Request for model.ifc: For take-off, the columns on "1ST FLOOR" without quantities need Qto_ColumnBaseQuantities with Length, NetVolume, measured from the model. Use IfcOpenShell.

First a look at what the model holds.

```python
import ifcopenshell
import ifcopenshell.util.element
import ifcopenshell.util.unit

model = ifcopenshell.open("model.ifc")
print(model.schema)
for unit_type in ("LENGTHUNIT", "AREAUNIT", "VOLUMEUNIT"):
    print(unit_type, ifcopenshell.util.unit.calculate_unit_scale(model, unit_type))
storey = next(s for s in model.by_type("IfcBuildingStorey") if s.Name == "1ST FLOOR")
columns = [e for e in ifcopenshell.util.element.get_decomposition(storey) if e.is_a("IfcColumn")]
for e in sorted(columns, key=lambda e: e.id()):
    print(e.id(), e.is_a(), e.Name, list(ifcopenshell.util.element.get_psets(e, qtos_only=True)), sep=" | ")
```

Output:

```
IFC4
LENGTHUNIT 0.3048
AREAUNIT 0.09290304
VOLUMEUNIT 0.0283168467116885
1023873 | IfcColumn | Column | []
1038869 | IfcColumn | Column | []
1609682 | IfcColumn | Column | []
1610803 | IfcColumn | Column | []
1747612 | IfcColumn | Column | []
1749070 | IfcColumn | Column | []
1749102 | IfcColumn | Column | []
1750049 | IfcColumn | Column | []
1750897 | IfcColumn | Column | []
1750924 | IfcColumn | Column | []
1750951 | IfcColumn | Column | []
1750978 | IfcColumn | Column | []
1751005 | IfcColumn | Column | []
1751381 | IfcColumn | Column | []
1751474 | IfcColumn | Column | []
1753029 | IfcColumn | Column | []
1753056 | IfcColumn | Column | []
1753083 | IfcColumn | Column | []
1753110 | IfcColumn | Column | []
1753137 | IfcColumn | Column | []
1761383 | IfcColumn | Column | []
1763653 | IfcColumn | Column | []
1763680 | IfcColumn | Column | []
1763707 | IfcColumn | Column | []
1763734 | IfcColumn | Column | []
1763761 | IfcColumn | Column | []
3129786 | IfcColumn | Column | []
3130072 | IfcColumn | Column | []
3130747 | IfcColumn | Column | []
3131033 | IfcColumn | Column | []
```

```python
import ifcopenshell
import ifcopenshell.api.pset
import ifcopenshell.geom
import ifcopenshell.util.element
import ifcopenshell.util.shape
import ifcopenshell.util.unit

model = ifcopenshell.open("model.ifc")
unit_scale = ifcopenshell.util.unit.calculate_unit_scale(model)
volume_scale = ifcopenshell.util.unit.calculate_unit_scale(model, "VOLUMEUNIT")
settings = ifcopenshell.geom.settings()

storey = next(s for s in model.by_type("IfcBuildingStorey") if s.Name == "1ST FLOOR")
columns = [e for e in ifcopenshell.util.element.get_decomposition(storey) if e.is_a("IfcColumn")]

for e in sorted(columns, key=lambda e: e.id()):
    if ifcopenshell.util.element.get_psets(e, qtos_only=True, should_inherit=False):
        continue
    # Geometry comes back in metres, in the element's own axes.
    shape = ifcopenshell.geom.create_shape(settings, e)
    values = {
        "Length": ifcopenshell.util.shape.get_z(shape.geometry) / unit_scale,
        "NetVolume": ifcopenshell.util.shape.get_volume(shape.geometry) / volume_scale,
    }
    qto = ifcopenshell.api.pset.add_qto(model, product=e, name="Qto_ColumnBaseQuantities")
    ifcopenshell.api.pset.edit_qto(model, qto=qto, properties=values)
    print(e.id(), {k: round(v, 3) for k, v in values.items()})

model.write("model_edited.ifc")
```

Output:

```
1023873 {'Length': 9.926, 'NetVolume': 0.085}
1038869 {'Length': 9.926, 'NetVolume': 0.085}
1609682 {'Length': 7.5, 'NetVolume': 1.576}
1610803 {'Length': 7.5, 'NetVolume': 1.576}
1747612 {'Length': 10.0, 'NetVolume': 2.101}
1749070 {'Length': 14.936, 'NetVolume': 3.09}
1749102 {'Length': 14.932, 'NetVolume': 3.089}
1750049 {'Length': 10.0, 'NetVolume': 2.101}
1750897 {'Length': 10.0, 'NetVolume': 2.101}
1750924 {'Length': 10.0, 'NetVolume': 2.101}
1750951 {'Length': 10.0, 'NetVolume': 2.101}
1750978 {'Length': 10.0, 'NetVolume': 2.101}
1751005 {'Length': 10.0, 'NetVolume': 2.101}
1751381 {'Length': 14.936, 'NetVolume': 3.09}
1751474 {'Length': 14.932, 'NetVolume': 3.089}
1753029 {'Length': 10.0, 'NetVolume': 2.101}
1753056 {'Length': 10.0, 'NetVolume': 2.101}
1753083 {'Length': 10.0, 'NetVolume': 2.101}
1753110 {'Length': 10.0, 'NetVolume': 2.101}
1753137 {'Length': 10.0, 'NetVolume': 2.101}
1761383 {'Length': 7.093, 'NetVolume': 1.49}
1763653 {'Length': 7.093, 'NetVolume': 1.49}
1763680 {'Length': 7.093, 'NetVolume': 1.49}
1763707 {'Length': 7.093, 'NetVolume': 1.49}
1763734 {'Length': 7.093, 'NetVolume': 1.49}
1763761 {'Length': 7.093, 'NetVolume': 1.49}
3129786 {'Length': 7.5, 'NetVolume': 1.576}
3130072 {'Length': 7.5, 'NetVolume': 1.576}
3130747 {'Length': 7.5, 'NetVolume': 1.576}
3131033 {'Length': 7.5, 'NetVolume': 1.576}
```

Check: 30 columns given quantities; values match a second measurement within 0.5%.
